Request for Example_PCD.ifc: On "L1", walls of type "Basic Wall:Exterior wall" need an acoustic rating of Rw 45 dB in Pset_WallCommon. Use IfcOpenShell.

First a look at what the model holds.

```python
import ifcopenshell
import ifcopenshell.util.element

model = ifcopenshell.open("Example_PCD.ifc")
print(model.schema)
storey = next(s for s in model.by_type("IfcBuildingStorey") if s.Name == "L1")
walls = [e for e in ifcopenshell.util.element.get_decomposition(storey) if e.is_a("IfcWall")]
seen = {}
for e in walls:
    element_type = ifcopenshell.util.element.get_type(e)
    key = (element_type.Name if element_type != e and element_type else None, ifcopenshell.util.element.get_pset(e, "Pset_WallCommon", "AcousticRating"))
    seen[key] = seen.get(key, 0) + 1
for (name, value), count in sorted(seen.items(), key=str):
    print(count, "x", name, "|", value)
```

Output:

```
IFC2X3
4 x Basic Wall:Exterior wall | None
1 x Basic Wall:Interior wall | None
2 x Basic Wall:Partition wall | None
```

```python
import ifcopenshell
import ifcopenshell.api.pset
import ifcopenshell.util.element

model = ifcopenshell.open("Example_PCD.ifc")

storey = next(s for s in model.by_type("IfcBuildingStorey") if s.Name == "L1")
walls = [e for e in ifcopenshell.util.element.get_decomposition(storey) if e.is_a("IfcWall")]

count = 0
for e in walls:
    element_type = ifcopenshell.util.element.get_type(e)
    if element_type in (None, e) or element_type.Name != "Basic Wall:Exterior wall":
        continue
    # add_pset returns the element's existing set when there is one.
    pset = ifcopenshell.api.pset.add_pset(model, product=e, name="Pset_WallCommon")
    ifcopenshell.api.pset.edit_pset(model, pset=pset, properties={"AcousticRating": "Rw 45 dB"})
    count += 1

print(count, "walls updated")

model.write("Example_PCD_v2.ifc")
```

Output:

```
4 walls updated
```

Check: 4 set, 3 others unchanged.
